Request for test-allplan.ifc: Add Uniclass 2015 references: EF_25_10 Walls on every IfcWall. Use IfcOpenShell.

First a look at what the model holds.

```python
import ifcopenshell

model = ifcopenshell.open("test-allplan.ifc")
print(model.schema)
print("classifications:", [c.Name for c in model.by_type("IfcClassification")])
for ifc_class in ("IfcDoor", "IfcRoof", "IfcStair", "IfcWall", "IfcWindow"):
    print(ifc_class, len(model.by_type(ifc_class)))
```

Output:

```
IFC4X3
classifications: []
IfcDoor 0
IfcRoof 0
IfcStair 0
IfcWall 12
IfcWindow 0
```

```python
import ifcopenshell
import ifcopenshell.api.classification

model = ifcopenshell.open("test-allplan.ifc")

system = ifcopenshell.api.classification.add_classification(model, classification="Uniclass 2015")

codes = {
    "IfcWall": ("EF_25_10", "Walls"),
}
for ifc_class, (code, name) in codes.items():
    products = model.by_type(ifc_class)
    ifcopenshell.api.classification.add_reference(
        model, products=products, classification=system, identification=code, name=name
    )
    print(code, len(products))

model.write("test-allplan_rev.ifc")
```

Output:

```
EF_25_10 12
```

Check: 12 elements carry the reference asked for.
